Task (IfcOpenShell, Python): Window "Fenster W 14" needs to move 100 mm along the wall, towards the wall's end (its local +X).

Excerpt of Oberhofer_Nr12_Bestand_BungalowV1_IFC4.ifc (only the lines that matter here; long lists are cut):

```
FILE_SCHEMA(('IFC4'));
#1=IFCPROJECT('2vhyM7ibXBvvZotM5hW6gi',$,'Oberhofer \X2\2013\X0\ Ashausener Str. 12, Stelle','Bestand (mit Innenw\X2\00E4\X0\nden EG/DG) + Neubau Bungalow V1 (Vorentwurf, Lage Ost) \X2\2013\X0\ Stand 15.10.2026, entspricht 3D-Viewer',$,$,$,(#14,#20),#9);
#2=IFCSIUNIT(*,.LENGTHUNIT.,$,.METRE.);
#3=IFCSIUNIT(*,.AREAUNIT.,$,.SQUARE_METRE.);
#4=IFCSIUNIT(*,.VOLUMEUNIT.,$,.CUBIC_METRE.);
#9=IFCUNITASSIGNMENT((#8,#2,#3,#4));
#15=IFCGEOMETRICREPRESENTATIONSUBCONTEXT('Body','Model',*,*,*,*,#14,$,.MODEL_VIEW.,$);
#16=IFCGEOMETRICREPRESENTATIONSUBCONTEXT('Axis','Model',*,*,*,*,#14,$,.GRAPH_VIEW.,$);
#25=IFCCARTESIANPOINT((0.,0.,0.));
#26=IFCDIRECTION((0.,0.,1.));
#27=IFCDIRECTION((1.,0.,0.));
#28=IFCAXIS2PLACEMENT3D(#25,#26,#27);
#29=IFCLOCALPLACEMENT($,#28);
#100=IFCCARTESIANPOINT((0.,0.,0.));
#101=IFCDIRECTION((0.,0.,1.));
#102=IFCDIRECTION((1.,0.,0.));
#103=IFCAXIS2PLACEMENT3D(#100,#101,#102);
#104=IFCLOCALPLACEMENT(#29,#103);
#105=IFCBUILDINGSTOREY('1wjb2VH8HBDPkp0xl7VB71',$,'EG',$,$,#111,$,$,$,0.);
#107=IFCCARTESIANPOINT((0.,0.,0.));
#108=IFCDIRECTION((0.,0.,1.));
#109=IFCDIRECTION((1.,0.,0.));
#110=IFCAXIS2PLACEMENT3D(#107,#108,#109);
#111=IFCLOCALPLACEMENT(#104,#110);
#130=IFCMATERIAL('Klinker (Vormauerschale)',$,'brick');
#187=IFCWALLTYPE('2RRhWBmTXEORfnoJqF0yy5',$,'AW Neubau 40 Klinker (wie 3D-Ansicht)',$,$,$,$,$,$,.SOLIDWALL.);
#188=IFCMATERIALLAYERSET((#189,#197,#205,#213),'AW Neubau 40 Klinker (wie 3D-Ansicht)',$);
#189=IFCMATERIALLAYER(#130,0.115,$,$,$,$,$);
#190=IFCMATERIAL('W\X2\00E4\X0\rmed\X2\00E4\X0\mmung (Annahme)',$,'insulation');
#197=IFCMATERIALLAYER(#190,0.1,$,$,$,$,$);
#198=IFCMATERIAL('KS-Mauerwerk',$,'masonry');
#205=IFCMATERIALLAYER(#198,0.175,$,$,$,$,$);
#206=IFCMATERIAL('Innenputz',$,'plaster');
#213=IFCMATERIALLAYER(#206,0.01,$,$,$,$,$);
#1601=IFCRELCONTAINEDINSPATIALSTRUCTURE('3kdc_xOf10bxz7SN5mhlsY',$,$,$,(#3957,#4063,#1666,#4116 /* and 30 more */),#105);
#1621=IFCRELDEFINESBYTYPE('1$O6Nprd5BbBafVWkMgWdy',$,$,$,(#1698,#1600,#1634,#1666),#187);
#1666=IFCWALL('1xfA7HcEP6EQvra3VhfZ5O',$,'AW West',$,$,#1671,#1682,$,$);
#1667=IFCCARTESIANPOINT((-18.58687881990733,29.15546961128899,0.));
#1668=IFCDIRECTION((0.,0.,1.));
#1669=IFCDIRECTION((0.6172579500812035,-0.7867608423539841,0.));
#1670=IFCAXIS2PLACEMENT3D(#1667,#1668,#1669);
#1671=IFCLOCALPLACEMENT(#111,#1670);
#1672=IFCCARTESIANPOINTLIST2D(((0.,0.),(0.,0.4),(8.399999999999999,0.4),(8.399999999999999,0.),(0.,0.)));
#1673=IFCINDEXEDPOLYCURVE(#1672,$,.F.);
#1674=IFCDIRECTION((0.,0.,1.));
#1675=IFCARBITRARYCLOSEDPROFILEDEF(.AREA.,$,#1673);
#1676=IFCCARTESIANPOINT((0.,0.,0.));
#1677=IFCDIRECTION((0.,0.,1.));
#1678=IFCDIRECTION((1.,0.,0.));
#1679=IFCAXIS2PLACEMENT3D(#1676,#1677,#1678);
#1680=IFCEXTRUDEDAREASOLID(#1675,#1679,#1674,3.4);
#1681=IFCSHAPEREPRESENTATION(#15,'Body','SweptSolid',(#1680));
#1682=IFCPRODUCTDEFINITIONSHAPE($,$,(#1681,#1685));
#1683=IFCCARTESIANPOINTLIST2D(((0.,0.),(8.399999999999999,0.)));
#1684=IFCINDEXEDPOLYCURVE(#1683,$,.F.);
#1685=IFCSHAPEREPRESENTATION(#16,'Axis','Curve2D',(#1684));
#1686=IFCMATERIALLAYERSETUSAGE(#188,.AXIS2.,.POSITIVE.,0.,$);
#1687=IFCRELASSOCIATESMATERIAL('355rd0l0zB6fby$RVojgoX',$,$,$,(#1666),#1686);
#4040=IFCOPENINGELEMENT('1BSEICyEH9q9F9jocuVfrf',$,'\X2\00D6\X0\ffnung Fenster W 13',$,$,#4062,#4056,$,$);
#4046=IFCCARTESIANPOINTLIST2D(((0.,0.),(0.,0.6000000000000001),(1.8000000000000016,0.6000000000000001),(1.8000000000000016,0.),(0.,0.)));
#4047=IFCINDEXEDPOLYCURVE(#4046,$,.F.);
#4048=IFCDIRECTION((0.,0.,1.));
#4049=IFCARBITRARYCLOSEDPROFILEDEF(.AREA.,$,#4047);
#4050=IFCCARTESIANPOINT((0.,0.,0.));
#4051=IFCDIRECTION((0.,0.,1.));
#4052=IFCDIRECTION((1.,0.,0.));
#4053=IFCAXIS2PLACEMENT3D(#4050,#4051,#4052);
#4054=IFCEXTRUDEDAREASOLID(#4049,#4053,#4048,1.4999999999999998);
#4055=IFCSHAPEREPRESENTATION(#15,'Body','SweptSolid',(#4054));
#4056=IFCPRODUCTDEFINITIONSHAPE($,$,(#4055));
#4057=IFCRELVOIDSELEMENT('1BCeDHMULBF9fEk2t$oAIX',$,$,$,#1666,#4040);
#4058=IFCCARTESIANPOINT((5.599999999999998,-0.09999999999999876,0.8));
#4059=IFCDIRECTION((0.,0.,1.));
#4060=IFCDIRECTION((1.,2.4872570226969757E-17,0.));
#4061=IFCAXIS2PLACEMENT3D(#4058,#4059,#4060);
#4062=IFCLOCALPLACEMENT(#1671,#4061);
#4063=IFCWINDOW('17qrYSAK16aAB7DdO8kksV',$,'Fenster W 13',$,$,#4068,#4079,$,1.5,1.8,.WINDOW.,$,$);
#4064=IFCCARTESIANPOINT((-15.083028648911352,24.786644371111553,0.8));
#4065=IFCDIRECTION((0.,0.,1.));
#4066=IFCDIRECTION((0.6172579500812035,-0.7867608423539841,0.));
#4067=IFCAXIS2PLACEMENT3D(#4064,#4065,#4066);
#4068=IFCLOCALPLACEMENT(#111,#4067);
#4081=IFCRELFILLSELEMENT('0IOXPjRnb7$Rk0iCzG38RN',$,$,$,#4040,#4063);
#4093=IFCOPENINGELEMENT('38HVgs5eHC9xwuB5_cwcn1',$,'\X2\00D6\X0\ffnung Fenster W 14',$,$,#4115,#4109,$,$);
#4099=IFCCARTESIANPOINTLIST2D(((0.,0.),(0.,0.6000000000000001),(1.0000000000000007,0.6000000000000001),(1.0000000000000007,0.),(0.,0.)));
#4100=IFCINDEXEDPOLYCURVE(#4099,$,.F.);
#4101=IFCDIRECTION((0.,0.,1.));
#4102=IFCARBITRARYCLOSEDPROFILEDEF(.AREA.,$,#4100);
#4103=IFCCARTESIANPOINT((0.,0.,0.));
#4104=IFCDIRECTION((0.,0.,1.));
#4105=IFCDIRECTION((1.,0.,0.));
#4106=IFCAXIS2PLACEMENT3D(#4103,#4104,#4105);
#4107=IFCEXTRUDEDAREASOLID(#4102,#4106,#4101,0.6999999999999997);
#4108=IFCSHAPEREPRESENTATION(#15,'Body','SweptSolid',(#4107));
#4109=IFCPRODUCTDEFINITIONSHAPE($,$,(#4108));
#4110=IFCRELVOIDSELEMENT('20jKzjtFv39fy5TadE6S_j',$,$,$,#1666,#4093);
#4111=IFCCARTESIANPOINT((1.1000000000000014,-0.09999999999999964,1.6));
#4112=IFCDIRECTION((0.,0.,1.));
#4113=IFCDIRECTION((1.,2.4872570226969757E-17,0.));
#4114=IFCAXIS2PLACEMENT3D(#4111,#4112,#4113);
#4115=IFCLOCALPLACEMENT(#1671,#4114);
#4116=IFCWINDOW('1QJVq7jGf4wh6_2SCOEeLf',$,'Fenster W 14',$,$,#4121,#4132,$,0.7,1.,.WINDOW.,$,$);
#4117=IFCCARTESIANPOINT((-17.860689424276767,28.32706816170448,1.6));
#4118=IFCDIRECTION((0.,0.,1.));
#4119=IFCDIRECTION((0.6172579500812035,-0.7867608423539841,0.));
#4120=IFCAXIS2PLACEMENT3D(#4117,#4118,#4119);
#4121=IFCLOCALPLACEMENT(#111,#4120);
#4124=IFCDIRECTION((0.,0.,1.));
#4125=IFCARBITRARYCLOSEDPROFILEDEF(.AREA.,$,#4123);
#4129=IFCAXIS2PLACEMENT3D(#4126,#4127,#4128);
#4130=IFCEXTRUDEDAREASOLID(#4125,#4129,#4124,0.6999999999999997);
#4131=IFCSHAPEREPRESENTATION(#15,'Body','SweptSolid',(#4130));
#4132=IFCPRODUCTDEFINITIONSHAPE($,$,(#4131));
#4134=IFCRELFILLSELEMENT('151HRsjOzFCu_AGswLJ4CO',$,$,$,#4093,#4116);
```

```python
import ifcopenshell
import ifcopenshell.api.geometry
import ifcopenshell.util.placement
import ifcopenshell.util.unit

model = ifcopenshell.open("Oberhofer_Nr12_Bestand_BungalowV1_IFC4.ifc")
unit_scale = ifcopenshell.util.unit.calculate_unit_scale(model)

window = model.by_guid("1QJVq7jGf4wh6_2SCOEeLf")
opening = window.FillsVoids[0].RelatingOpeningElement
wall = opening.VoidsElements[0].RelatingBuildingElement

wall_matrix = ifcopenshell.util.placement.get_local_placement(wall.ObjectPlacement)
shift = wall_matrix[:3, 0] * 0.1 / unit_scale
before = ifcopenshell.util.placement.get_local_placement(window.ObjectPlacement)[:3, 3].copy()

# The window is not placed relative to its opening, so move both.
for product in (opening, window):
    matrix = ifcopenshell.util.placement.get_local_placement(product.ObjectPlacement)
    matrix[:3, 3] += shift
    ifcopenshell.api.geometry.edit_object_placement(model, product=product, matrix=matrix, is_si=False)

after = ifcopenshell.util.placement.get_local_placement(window.ObjectPlacement)[:3, 3]
print("window moved by", (after - before).round(3) + 0.0)

model.write("Oberhofer_Nr12_Bestand_BungalowV1_IFC4_edited.ifc")
```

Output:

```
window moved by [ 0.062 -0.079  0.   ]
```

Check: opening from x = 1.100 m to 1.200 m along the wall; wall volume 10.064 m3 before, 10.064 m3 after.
